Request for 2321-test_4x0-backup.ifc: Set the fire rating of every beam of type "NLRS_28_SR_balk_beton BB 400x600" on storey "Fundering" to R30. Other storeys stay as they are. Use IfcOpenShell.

First a look at what the model holds.

```python
import ifcopenshell
import ifcopenshell.util.element

model = ifcopenshell.open("2321-test_4x0-backup.ifc")
print(model.schema)
storey = next(s for s in model.by_type("IfcBuildingStorey") if s.Name == "Fundering")
beams = [e for e in ifcopenshell.util.element.get_decomposition(storey) if e.is_a("IfcBeam")]
seen = {}
for e in beams:
    element_type = ifcopenshell.util.element.get_type(e)
    key = (element_type.Name if element_type != e and element_type else None, ifcopenshell.util.element.get_pset(e, "Pset_BeamCommon", "FireRating"))
    seen[key] = seen.get(key, 0) + 1
for (name, value), count in sorted(seen.items(), key=str):
    print(count, "x", name, "|", value)
```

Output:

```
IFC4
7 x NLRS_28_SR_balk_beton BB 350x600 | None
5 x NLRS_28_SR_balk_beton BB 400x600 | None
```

```python
import ifcopenshell
import ifcopenshell.api.pset
import ifcopenshell.util.element

model = ifcopenshell.open("2321-test_4x0-backup.ifc")

storey = next(s for s in model.by_type("IfcBuildingStorey") if s.Name == "Fundering")
beams = [e for e in ifcopenshell.util.element.get_decomposition(storey) if e.is_a("IfcBeam")]

count = 0
for e in beams:
    element_type = ifcopenshell.util.element.get_type(e)
    if element_type in (None, e) or element_type.Name != "NLRS_28_SR_balk_beton BB 400x600":
        continue
    # add_pset returns the element's existing set when there is one.
    pset = ifcopenshell.api.pset.add_pset(model, product=e, name="Pset_BeamCommon")
    ifcopenshell.api.pset.edit_pset(model, pset=pset, properties={"FireRating": "R30"})
    count += 1

print(count, "beams updated")

model.write("2321-test_4x0-backup_edited.ifc")
```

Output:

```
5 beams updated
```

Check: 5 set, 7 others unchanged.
